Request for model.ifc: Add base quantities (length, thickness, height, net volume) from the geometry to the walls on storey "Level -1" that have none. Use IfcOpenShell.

First a look at what the model holds.

```python
import ifcopenshell
import ifcopenshell.util.element
import ifcopenshell.util.unit

model = ifcopenshell.open("model.ifc")
print(model.schema)
for unit_type in ("LENGTHUNIT", "AREAUNIT", "VOLUMEUNIT"):
    print(unit_type, ifcopenshell.util.unit.calculate_unit_scale(model, unit_type))
storey = next(s for s in model.by_type("IfcBuildingStorey") if s.Name == "Level -1")
walls = [e for e in ifcopenshell.util.element.get_decomposition(storey) if e.is_a("IfcWall")]
for e in sorted(walls, key=lambda e: e.id()):
    print(e.id(), e.is_a(), e.Name, list(ifcopenshell.util.element.get_psets(e, qtos_only=True)), sep=" | ")
```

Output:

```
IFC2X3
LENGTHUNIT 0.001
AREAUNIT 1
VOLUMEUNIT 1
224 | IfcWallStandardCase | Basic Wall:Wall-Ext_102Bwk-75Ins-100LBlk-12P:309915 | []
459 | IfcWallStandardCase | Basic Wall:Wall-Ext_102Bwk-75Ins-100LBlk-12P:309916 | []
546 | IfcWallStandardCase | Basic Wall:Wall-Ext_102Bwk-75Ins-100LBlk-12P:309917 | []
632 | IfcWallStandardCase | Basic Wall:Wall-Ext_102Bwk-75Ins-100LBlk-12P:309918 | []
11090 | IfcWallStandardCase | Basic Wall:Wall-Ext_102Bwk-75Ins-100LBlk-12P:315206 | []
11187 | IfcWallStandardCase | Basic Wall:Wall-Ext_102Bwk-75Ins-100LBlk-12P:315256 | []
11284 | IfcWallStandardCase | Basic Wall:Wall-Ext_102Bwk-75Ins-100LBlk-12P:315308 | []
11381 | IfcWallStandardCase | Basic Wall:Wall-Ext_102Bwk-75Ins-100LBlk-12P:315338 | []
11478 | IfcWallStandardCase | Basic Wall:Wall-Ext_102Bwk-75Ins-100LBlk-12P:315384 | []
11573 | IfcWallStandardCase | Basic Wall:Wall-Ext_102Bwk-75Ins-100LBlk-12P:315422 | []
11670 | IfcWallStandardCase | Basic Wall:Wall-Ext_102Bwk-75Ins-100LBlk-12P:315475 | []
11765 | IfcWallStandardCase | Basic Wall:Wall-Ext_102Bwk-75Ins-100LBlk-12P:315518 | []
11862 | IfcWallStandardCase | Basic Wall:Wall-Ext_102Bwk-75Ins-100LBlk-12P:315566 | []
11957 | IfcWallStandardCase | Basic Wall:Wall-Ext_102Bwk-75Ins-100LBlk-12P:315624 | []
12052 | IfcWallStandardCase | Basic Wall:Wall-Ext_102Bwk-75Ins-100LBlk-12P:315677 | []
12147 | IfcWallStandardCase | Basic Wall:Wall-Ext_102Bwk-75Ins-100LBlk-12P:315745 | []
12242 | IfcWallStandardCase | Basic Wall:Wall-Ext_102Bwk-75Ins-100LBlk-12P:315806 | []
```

```python
import ifcopenshell
import ifcopenshell.api.pset
import ifcopenshell.geom
import ifcopenshell.util.element
import ifcopenshell.util.shape
import ifcopenshell.util.unit

model = ifcopenshell.open("model.ifc")
unit_scale = ifcopenshell.util.unit.calculate_unit_scale(model)
volume_scale = ifcopenshell.util.unit.calculate_unit_scale(model, "VOLUMEUNIT")
settings = ifcopenshell.geom.settings()

storey = next(s for s in model.by_type("IfcBuildingStorey") if s.Name == "Level -1")
walls = [e for e in ifcopenshell.util.element.get_decomposition(storey) if e.is_a("IfcWall")]

for e in sorted(walls, key=lambda e: e.id()):
    if ifcopenshell.util.element.get_psets(e, qtos_only=True, should_inherit=False):
        continue
    # Geometry comes back in metres, in the element's own axes.
    shape = ifcopenshell.geom.create_shape(settings, e)
    values = {
        "Length": ifcopenshell.util.shape.get_x(shape.geometry) / unit_scale,
        "Width": ifcopenshell.util.shape.get_y(shape.geometry) / unit_scale,
        "Height": ifcopenshell.util.shape.get_z(shape.geometry) / unit_scale,
        "NetVolume": ifcopenshell.util.shape.get_volume(shape.geometry) / volume_scale,
    }
    qto = ifcopenshell.api.pset.add_qto(model, product=e, name="BaseQuantities")
    ifcopenshell.api.pset.edit_qto(model, qto=qto, properties=values)
    print(e.id(), {k: round(v, 3) for k, v in values.items()})

model.write("model_updated.ifc")
```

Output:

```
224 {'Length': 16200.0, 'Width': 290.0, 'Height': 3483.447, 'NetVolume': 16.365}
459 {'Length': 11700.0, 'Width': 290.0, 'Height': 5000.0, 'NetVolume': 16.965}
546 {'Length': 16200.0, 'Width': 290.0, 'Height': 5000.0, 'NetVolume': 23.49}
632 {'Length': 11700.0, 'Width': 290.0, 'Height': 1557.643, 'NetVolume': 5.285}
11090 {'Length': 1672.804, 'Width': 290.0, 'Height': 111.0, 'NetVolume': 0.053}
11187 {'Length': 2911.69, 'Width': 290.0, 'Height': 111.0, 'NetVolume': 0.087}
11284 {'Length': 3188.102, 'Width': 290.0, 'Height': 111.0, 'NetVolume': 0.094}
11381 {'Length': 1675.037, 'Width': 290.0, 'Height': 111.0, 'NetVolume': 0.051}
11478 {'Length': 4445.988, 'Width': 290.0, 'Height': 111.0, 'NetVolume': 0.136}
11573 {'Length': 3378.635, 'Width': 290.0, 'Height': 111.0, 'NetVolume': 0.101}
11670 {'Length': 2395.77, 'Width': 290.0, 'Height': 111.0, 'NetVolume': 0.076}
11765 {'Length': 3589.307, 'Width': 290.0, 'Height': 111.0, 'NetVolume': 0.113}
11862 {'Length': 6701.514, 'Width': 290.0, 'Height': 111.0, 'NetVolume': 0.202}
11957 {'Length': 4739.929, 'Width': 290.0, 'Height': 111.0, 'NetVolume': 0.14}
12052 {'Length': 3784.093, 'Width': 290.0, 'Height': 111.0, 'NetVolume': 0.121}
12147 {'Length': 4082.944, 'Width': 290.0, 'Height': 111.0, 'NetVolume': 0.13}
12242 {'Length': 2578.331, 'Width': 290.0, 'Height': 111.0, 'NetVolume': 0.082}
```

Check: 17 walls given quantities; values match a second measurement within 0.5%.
